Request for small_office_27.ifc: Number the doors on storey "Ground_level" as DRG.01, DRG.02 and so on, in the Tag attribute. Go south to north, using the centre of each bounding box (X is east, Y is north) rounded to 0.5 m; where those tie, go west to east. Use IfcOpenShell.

First a look at what the model holds.

```python
import ifcopenshell
import ifcopenshell.util.element
import ifcopenshell.util.placement

model = ifcopenshell.open("small_office_27.ifc")
print(model.schema)
storey = next(s for s in model.by_type("IfcBuildingStorey") if s.Name == "Ground_level")
doors = [e for e in ifcopenshell.util.element.get_decomposition(storey) if e.is_a("IfcDoor")]
for e in sorted(doors, key=lambda e: e.id()):
    origin = ifcopenshell.util.placement.get_local_placement(e.ObjectPlacement)[:3, 3]
    print(e.id(), e.Tag, e.Name, origin.round(2) + 0.0, sep=" | ")
```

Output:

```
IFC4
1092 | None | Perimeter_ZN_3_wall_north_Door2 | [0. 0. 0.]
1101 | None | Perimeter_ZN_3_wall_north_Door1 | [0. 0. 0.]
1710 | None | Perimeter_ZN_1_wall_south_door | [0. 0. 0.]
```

```python
import ifcopenshell
import ifcopenshell.geom
import ifcopenshell.util.element
import ifcopenshell.util.shape

model = ifcopenshell.open("small_office_27.ifc")
settings = ifcopenshell.geom.settings()
settings.set("use-world-coords", True)


def centre(element):
    shape = ifcopenshell.geom.create_shape(settings, element)
    return ifcopenshell.util.shape.get_bbox_centroid(shape.geometry)


storey = next(s for s in model.by_type("IfcBuildingStorey") if s.Name == "Ground_level")
doors = [e for e in ifcopenshell.util.element.get_decomposition(storey) if e.is_a("IfcDoor")]

# Insertion points can sit at a corner or the storey origin, so sort by the geometry (in metres).
centres = {e: centre(e) for e in doors}
doors.sort(key=lambda e: (round(centres[e][1] / 0.5), centres[e][0]))

for i, e in enumerate(doors, start=1):
    number = f"DRG.{i:02d}"
    e.Tag = number
    print(e.id(), number)

model.write("small_office_27_edited.ifc")
```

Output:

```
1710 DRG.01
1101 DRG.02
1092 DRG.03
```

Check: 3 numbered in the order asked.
